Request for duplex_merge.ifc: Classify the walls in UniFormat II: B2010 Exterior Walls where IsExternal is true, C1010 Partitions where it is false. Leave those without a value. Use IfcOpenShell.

First a look at what the model holds.

```python
import ifcopenshell
import ifcopenshell.util.element

model = ifcopenshell.open("duplex_merge.ifc")
print(model.schema)
print("classifications:", [c.Name for c in model.by_type("IfcClassification")])
values = [ifcopenshell.util.element.get_pset(e, "Pset_WallCommon", "IsExternal") for e in model.by_type("IfcWall")]
for value in (True, False, None):
    print("IsExternal", value, values.count(value))
```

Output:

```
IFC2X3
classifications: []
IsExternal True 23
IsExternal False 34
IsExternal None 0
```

```python
import ifcopenshell
import ifcopenshell.api.classification
import ifcopenshell.util.element

model = ifcopenshell.open("duplex_merge.ifc")

# IFC2X3 requires Source and Edition and has no link from the project to the system.
system = model.create_entity("IfcClassification", Source="ASTM", Edition="E1557", Name="UniFormat II")

walls = model.by_type("IfcWall")
external = {e: ifcopenshell.util.element.get_pset(e, "Pset_WallCommon", "IsExternal") for e in walls}
for flag, code, name in ((True, "B2010", "Exterior Walls"), (False, "C1010", "Partitions")):
    products = [e for e in walls if external[e] is flag]
    ifcopenshell.api.classification.add_reference(
        model, products=products, classification=system, identification=code, name=name
    )
    print(code, len(products))

model.write("duplex_merge-out.ifc")
```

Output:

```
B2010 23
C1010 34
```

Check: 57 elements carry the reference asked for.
